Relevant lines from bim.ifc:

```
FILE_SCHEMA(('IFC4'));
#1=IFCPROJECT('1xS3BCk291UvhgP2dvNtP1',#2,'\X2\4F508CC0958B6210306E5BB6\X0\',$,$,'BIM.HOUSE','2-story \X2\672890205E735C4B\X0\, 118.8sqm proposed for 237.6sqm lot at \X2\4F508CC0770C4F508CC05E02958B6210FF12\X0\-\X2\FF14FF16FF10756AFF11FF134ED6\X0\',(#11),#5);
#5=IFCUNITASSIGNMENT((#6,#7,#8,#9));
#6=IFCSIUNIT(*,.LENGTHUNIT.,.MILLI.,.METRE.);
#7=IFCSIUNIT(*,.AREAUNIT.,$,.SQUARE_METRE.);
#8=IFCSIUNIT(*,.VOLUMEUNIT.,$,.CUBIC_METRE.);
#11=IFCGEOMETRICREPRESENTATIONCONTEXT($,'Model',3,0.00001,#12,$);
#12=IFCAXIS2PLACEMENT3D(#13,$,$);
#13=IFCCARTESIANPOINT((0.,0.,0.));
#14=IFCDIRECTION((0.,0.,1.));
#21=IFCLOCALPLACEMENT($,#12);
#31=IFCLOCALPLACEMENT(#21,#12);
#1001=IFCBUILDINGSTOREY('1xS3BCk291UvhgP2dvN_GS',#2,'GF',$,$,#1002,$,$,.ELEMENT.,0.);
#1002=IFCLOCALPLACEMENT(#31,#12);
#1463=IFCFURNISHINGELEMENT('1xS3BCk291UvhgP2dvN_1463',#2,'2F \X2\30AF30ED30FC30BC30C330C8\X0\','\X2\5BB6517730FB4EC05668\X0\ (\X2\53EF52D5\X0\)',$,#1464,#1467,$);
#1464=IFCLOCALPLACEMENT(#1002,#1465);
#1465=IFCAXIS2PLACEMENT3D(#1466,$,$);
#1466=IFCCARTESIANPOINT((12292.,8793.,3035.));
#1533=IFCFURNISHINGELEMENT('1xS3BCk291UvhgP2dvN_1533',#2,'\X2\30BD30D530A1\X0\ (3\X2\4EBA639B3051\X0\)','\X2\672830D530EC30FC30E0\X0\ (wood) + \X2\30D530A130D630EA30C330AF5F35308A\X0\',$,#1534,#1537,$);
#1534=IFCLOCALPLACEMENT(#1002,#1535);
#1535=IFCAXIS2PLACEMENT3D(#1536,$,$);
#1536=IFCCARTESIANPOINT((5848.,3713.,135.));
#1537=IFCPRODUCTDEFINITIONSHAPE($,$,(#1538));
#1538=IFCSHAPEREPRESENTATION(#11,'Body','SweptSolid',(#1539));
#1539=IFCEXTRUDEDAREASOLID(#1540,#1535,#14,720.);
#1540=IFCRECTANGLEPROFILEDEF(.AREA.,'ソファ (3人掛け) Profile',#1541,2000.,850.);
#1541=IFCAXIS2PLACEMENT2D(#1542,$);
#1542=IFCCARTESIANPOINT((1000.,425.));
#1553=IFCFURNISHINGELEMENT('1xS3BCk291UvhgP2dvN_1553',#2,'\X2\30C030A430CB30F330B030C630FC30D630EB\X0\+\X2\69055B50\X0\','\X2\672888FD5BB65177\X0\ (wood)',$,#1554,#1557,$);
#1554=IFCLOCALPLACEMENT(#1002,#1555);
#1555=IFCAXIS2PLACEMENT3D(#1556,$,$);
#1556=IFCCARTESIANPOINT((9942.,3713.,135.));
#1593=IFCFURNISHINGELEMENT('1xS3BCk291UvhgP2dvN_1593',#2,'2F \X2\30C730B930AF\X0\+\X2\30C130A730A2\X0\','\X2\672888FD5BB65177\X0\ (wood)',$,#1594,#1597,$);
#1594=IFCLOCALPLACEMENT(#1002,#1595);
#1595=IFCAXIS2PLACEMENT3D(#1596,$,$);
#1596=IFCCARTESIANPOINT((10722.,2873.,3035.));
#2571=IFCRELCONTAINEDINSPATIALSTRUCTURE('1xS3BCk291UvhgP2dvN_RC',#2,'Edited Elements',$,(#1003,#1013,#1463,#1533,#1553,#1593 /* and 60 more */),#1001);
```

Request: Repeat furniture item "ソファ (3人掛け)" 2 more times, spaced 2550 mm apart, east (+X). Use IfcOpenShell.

```python
import numpy as np
import ifcopenshell
import ifcopenshell.api.geometry
import ifcopenshell.api.root
import ifcopenshell.util.element
import ifcopenshell.util.placement
import ifcopenshell.util.unit

model = ifcopenshell.open("bim.ifc")
unit_scale = ifcopenshell.util.unit.calculate_unit_scale(model)


def reuse_history(source, copy):
    """copy_class also copies each property set's owner history, people and application; keep the originals."""
    for rel in copy.IsDefinedBy:
        if rel.is_a("IfcRelDefinesByProperties") and (history := rel.RelatingPropertyDefinition.OwnerHistory):
            rel.RelatingPropertyDefinition.OwnerHistory = source.OwnerHistory
            ifcopenshell.util.element.remove_deep2(model, history)


source = model.by_guid("1xS3BCk291UvhgP2dvN_1533")
base = ifcopenshell.util.placement.get_local_placement(source.ObjectPlacement)
step = np.array([1.0, 0.0, 0.0]) * 2.55 / unit_scale

for i in range(1, 3):
    copy = ifcopenshell.api.root.copy_class(model, product=source)
    copy.Representation = ifcopenshell.util.element.copy_deep(
        model, source.Representation, exclude=["IfcGeometricRepresentationContext", "IfcRepresentationMap"]
    )
    reuse_history(source, copy)
    matrix = base.copy()
    matrix[:3, 3] += i * step
    print("added at", matrix[:3, 3].round(3) + 0.0)
    ifcopenshell.api.geometry.edit_object_placement(model, product=copy, matrix=matrix, is_si=False)

model.write("bim-out.ifc")
```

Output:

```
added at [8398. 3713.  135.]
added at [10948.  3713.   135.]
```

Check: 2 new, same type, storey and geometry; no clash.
